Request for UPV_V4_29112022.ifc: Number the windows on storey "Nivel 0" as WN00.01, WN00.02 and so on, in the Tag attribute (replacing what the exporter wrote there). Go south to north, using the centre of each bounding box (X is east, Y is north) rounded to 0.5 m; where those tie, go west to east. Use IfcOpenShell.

First a look at what the model holds.

```python
import ifcopenshell
import ifcopenshell.util.element
import ifcopenshell.util.placement

model = ifcopenshell.open("UPV_V4_29112022.ifc")
print(model.schema)
storey = next(s for s in model.by_type("IfcBuildingStorey") if s.Name == "Nivel 0")
windows = [e for e in ifcopenshell.util.element.get_decomposition(storey) if e.is_a("IfcWindow")]
for e in sorted(windows, key=lambda e: e.id()):
    origin = ifcopenshell.util.placement.get_local_placement(e.ObjectPlacement)[:3, 3]
    print(e.id(), e.Tag, e.Name, origin.round(2) + 0.0, sep=" | ")
```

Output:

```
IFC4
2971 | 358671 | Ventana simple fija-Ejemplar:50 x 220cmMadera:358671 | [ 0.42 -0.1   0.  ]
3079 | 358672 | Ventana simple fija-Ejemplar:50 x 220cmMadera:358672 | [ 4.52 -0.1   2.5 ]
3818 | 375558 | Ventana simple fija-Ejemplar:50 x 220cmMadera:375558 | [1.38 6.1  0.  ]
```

```python
import ifcopenshell
import ifcopenshell.geom
import ifcopenshell.util.element
import ifcopenshell.util.shape

model = ifcopenshell.open("UPV_V4_29112022.ifc")
settings = ifcopenshell.geom.settings()
settings.set("use-world-coords", True)


def centre(element):
    shape = ifcopenshell.geom.create_shape(settings, element)
    return ifcopenshell.util.shape.get_bbox_centroid(shape.geometry)


storey = next(s for s in model.by_type("IfcBuildingStorey") if s.Name == "Nivel 0")
windows = [e for e in ifcopenshell.util.element.get_decomposition(storey) if e.is_a("IfcWindow")]

# Insertion points can sit at a corner or the storey origin, so sort by the geometry (in metres).
centres = {e: centre(e) for e in windows}
windows.sort(key=lambda e: (round(centres[e][1] / 0.5), centres[e][0]))

for i, e in enumerate(windows, start=1):
    number = f"WN00.{i:02d}"
    e.Tag = number
    print(e.id(), number)

model.write("UPV_V4_29112022_v2.ifc")
```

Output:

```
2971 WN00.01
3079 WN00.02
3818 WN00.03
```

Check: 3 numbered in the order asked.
